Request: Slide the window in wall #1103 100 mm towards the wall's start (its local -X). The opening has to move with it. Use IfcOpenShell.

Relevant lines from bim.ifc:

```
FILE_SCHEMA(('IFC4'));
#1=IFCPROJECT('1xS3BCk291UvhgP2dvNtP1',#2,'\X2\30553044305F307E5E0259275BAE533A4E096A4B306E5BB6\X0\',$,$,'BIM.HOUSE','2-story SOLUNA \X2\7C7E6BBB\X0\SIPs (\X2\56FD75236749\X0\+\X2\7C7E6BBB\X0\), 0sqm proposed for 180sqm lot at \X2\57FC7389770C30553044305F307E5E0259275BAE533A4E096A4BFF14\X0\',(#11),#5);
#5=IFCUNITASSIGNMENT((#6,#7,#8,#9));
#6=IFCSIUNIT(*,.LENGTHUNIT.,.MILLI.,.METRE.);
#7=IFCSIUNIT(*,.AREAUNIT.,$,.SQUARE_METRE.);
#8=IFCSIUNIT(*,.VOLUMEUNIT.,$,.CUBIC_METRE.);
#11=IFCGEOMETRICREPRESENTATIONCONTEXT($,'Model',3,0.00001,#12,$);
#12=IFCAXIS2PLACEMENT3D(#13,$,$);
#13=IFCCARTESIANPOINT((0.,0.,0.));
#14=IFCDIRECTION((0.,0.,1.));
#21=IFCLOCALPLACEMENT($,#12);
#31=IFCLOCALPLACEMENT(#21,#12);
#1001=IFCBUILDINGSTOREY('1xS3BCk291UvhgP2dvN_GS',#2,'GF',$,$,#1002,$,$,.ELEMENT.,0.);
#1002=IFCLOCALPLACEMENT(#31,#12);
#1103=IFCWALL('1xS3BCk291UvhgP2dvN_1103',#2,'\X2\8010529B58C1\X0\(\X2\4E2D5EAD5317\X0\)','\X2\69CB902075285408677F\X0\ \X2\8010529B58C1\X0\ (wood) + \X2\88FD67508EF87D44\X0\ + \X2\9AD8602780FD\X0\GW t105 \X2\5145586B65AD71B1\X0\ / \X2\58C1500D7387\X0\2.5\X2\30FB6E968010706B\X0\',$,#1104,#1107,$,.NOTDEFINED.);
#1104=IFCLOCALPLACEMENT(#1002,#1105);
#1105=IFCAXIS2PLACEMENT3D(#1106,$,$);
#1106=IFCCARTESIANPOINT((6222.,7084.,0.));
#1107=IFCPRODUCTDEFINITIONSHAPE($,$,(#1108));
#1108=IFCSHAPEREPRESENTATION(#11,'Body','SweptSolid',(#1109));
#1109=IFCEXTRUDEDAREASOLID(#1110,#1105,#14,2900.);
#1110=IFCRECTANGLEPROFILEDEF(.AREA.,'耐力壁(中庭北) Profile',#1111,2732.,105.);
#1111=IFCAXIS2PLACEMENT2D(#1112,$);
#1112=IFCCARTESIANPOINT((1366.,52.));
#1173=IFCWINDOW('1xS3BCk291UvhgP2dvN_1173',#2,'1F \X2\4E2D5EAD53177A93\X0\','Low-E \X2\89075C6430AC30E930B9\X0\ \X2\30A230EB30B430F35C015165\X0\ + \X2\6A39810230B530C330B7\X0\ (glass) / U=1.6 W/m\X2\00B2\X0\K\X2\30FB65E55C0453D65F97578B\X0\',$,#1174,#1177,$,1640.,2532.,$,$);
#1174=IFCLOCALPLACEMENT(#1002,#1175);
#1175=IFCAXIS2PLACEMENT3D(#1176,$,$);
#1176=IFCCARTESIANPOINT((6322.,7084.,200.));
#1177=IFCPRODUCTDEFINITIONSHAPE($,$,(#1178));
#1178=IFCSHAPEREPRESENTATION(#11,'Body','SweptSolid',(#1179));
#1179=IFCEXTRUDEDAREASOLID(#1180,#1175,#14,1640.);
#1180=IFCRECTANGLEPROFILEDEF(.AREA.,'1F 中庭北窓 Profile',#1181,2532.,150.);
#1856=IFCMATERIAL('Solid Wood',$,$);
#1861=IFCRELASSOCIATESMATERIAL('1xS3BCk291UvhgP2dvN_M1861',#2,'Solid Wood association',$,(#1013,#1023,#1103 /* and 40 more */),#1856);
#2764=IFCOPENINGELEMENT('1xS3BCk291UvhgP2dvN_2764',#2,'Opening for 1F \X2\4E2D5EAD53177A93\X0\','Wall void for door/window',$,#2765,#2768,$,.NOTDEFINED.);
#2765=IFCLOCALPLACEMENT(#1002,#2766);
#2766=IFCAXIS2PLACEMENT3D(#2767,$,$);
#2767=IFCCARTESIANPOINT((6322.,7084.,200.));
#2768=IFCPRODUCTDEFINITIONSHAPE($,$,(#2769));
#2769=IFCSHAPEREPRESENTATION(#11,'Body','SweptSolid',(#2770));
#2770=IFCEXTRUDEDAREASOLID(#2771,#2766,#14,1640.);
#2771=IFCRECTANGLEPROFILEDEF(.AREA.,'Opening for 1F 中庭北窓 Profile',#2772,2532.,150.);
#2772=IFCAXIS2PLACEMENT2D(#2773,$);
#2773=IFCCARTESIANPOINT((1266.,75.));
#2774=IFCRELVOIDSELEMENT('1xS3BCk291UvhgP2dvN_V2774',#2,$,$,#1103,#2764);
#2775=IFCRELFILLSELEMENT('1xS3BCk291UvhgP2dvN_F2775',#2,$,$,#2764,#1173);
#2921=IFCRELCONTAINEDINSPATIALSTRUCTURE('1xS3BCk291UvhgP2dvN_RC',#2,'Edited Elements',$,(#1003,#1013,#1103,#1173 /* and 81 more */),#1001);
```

```python
import ifcopenshell
import ifcopenshell.api.geometry
import ifcopenshell.util.placement

model = ifcopenshell.open("bim.ifc")

window = model.by_id(1173)
opening = window.FillsVoids[0].RelatingOpeningElement
wall = opening.VoidsElements[0].RelatingBuildingElement

wall_matrix = ifcopenshell.util.placement.get_local_placement(wall.ObjectPlacement)
shift = wall_matrix[:3, 0] * -100.0
before = ifcopenshell.util.placement.get_local_placement(window.ObjectPlacement)[:3, 3].copy()

# The window is not placed relative to its opening, so move both.
for product in (opening, window):
    matrix = ifcopenshell.util.placement.get_local_placement(product.ObjectPlacement)
    matrix[:3, 3] += shift
    ifcopenshell.api.geometry.edit_object_placement(model, product=product, matrix=matrix, is_si=False)

after = ifcopenshell.util.placement.get_local_placement(window.ObjectPlacement)[:3, 3]
print("window moved by", (after - before).round(3) + 0.0)

model.write("bim_edited.ifc")
```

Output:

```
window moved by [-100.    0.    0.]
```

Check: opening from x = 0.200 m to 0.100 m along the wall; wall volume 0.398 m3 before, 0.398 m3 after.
